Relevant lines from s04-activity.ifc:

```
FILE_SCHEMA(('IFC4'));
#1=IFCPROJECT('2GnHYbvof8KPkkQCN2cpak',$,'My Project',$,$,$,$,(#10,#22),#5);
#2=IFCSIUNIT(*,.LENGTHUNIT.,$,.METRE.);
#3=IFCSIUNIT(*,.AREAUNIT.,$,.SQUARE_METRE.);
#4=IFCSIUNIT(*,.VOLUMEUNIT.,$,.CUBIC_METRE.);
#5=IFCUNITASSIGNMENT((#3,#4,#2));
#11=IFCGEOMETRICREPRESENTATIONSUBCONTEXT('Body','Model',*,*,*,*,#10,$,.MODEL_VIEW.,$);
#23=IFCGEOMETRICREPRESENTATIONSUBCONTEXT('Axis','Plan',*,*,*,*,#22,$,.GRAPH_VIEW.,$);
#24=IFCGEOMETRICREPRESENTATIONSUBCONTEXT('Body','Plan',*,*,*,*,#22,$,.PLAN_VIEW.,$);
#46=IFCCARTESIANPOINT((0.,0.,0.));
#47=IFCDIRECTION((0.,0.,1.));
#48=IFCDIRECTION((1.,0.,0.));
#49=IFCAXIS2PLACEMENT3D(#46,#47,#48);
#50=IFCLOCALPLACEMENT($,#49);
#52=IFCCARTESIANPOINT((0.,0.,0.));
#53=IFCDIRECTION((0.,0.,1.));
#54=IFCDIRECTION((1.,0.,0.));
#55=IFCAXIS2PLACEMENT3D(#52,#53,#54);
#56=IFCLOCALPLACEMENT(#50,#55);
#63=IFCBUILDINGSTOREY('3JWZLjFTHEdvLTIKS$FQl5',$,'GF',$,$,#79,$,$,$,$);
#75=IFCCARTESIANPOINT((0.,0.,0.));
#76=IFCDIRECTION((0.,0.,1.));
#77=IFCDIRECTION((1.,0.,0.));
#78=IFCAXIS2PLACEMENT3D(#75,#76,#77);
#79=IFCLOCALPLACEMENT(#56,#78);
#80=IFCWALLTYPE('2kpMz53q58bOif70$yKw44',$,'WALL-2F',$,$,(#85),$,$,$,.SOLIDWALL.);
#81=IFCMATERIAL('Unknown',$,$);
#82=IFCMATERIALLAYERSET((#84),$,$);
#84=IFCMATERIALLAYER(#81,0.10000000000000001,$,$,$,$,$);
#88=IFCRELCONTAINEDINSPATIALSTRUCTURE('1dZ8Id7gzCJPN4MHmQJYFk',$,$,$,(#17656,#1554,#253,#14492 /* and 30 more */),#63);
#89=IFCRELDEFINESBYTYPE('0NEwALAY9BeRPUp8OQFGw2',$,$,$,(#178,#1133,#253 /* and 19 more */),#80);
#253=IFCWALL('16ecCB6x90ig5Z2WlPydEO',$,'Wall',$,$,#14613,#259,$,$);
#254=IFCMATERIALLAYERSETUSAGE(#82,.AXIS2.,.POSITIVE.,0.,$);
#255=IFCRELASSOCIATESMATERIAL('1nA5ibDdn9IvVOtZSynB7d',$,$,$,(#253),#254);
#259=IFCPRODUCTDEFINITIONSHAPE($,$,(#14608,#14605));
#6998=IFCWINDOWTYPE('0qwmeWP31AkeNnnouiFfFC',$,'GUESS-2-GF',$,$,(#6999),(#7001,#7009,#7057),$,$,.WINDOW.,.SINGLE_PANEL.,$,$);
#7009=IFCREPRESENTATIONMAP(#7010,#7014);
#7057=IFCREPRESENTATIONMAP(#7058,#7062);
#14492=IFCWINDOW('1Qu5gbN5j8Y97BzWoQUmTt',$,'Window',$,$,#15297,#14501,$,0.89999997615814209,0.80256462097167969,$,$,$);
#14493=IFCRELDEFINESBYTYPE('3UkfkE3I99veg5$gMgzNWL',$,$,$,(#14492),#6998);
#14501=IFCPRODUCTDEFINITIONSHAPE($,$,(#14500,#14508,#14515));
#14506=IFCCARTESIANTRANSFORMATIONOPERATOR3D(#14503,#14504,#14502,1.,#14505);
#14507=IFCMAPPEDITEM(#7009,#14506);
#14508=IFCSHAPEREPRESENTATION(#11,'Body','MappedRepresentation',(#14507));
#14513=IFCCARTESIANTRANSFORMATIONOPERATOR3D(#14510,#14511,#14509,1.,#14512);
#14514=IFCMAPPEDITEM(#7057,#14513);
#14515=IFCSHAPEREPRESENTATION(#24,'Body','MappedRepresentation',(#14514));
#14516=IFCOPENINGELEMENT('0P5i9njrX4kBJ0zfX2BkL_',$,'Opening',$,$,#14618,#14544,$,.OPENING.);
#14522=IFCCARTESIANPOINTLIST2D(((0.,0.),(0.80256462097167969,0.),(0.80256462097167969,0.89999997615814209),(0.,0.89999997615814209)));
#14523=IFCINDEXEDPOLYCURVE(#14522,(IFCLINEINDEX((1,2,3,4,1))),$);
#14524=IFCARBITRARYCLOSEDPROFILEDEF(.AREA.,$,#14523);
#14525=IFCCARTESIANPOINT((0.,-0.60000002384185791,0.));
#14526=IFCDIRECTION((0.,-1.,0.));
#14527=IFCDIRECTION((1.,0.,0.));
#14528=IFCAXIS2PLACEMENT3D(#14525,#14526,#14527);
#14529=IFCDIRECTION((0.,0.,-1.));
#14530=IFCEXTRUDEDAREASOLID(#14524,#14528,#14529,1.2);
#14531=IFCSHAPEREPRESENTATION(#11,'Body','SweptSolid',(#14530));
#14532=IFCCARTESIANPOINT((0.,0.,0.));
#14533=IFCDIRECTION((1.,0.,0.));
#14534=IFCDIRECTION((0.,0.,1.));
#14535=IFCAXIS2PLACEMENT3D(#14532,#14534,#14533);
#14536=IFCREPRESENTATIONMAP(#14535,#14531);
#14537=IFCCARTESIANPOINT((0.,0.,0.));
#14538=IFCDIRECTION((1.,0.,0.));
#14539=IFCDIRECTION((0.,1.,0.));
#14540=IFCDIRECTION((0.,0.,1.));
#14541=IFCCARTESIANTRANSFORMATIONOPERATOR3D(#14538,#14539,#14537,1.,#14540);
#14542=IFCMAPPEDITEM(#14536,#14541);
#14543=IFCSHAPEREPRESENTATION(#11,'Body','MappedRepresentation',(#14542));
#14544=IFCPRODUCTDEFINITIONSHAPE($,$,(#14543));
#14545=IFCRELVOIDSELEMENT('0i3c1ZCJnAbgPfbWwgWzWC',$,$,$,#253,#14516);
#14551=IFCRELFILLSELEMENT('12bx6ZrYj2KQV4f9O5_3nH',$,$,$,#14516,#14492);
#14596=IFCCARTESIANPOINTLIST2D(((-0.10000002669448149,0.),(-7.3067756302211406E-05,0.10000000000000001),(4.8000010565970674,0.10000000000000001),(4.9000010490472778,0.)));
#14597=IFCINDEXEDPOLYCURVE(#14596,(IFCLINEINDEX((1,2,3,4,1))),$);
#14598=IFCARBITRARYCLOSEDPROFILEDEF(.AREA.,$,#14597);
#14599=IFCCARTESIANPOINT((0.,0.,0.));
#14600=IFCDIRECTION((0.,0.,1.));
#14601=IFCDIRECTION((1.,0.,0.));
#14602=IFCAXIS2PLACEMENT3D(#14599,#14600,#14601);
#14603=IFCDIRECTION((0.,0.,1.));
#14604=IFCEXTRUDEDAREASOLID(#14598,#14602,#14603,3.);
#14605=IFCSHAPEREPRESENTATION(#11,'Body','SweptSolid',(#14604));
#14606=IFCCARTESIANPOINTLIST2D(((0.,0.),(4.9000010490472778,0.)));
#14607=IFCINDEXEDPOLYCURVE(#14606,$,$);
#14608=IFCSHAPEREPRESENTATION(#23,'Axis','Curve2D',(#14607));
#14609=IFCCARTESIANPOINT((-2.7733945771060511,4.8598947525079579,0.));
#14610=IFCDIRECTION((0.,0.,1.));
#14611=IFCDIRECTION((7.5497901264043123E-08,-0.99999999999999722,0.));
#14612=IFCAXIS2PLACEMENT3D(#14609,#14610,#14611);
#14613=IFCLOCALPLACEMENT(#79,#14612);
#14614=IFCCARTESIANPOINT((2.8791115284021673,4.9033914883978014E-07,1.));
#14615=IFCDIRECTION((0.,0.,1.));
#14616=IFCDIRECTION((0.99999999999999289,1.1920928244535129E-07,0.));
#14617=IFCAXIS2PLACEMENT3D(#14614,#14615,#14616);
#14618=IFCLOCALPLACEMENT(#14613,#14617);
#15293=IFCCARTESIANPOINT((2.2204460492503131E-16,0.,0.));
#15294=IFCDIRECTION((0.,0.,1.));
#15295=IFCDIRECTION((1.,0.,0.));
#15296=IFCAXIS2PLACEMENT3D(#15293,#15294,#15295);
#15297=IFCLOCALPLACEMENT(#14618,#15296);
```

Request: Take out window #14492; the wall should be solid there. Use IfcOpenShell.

```python
import ifcopenshell
import ifcopenshell.api.feature
import ifcopenshell.api.root
import ifcopenshell.geom
import ifcopenshell.util.shape

model = ifcopenshell.open("s04-activity.ifc")
settings = ifcopenshell.geom.settings()


def volume(element):
    """Net volume in cubic metres, openings subtracted."""
    shape = ifcopenshell.geom.create_shape(settings, element)
    return ifcopenshell.util.shape.get_volume(shape.geometry)


window = model.by_guid("1Qu5gbN5j8Y97BzWoQUmTt")
opening = window.FillsVoids[0].RelatingOpeningElement
wall = opening.VoidsElements[0].RelatingBuildingElement
before = volume(wall)

ifcopenshell.api.root.remove_product(model, product=window)
ifcopenshell.api.feature.remove_feature(model, feature=opening)

after = volume(wall)

print(f"wall volume {before:.3f} -> {after:.3f} m3")

model.write("s04-activity_edited.ifc")
```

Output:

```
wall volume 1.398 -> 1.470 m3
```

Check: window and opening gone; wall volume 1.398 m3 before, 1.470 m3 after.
